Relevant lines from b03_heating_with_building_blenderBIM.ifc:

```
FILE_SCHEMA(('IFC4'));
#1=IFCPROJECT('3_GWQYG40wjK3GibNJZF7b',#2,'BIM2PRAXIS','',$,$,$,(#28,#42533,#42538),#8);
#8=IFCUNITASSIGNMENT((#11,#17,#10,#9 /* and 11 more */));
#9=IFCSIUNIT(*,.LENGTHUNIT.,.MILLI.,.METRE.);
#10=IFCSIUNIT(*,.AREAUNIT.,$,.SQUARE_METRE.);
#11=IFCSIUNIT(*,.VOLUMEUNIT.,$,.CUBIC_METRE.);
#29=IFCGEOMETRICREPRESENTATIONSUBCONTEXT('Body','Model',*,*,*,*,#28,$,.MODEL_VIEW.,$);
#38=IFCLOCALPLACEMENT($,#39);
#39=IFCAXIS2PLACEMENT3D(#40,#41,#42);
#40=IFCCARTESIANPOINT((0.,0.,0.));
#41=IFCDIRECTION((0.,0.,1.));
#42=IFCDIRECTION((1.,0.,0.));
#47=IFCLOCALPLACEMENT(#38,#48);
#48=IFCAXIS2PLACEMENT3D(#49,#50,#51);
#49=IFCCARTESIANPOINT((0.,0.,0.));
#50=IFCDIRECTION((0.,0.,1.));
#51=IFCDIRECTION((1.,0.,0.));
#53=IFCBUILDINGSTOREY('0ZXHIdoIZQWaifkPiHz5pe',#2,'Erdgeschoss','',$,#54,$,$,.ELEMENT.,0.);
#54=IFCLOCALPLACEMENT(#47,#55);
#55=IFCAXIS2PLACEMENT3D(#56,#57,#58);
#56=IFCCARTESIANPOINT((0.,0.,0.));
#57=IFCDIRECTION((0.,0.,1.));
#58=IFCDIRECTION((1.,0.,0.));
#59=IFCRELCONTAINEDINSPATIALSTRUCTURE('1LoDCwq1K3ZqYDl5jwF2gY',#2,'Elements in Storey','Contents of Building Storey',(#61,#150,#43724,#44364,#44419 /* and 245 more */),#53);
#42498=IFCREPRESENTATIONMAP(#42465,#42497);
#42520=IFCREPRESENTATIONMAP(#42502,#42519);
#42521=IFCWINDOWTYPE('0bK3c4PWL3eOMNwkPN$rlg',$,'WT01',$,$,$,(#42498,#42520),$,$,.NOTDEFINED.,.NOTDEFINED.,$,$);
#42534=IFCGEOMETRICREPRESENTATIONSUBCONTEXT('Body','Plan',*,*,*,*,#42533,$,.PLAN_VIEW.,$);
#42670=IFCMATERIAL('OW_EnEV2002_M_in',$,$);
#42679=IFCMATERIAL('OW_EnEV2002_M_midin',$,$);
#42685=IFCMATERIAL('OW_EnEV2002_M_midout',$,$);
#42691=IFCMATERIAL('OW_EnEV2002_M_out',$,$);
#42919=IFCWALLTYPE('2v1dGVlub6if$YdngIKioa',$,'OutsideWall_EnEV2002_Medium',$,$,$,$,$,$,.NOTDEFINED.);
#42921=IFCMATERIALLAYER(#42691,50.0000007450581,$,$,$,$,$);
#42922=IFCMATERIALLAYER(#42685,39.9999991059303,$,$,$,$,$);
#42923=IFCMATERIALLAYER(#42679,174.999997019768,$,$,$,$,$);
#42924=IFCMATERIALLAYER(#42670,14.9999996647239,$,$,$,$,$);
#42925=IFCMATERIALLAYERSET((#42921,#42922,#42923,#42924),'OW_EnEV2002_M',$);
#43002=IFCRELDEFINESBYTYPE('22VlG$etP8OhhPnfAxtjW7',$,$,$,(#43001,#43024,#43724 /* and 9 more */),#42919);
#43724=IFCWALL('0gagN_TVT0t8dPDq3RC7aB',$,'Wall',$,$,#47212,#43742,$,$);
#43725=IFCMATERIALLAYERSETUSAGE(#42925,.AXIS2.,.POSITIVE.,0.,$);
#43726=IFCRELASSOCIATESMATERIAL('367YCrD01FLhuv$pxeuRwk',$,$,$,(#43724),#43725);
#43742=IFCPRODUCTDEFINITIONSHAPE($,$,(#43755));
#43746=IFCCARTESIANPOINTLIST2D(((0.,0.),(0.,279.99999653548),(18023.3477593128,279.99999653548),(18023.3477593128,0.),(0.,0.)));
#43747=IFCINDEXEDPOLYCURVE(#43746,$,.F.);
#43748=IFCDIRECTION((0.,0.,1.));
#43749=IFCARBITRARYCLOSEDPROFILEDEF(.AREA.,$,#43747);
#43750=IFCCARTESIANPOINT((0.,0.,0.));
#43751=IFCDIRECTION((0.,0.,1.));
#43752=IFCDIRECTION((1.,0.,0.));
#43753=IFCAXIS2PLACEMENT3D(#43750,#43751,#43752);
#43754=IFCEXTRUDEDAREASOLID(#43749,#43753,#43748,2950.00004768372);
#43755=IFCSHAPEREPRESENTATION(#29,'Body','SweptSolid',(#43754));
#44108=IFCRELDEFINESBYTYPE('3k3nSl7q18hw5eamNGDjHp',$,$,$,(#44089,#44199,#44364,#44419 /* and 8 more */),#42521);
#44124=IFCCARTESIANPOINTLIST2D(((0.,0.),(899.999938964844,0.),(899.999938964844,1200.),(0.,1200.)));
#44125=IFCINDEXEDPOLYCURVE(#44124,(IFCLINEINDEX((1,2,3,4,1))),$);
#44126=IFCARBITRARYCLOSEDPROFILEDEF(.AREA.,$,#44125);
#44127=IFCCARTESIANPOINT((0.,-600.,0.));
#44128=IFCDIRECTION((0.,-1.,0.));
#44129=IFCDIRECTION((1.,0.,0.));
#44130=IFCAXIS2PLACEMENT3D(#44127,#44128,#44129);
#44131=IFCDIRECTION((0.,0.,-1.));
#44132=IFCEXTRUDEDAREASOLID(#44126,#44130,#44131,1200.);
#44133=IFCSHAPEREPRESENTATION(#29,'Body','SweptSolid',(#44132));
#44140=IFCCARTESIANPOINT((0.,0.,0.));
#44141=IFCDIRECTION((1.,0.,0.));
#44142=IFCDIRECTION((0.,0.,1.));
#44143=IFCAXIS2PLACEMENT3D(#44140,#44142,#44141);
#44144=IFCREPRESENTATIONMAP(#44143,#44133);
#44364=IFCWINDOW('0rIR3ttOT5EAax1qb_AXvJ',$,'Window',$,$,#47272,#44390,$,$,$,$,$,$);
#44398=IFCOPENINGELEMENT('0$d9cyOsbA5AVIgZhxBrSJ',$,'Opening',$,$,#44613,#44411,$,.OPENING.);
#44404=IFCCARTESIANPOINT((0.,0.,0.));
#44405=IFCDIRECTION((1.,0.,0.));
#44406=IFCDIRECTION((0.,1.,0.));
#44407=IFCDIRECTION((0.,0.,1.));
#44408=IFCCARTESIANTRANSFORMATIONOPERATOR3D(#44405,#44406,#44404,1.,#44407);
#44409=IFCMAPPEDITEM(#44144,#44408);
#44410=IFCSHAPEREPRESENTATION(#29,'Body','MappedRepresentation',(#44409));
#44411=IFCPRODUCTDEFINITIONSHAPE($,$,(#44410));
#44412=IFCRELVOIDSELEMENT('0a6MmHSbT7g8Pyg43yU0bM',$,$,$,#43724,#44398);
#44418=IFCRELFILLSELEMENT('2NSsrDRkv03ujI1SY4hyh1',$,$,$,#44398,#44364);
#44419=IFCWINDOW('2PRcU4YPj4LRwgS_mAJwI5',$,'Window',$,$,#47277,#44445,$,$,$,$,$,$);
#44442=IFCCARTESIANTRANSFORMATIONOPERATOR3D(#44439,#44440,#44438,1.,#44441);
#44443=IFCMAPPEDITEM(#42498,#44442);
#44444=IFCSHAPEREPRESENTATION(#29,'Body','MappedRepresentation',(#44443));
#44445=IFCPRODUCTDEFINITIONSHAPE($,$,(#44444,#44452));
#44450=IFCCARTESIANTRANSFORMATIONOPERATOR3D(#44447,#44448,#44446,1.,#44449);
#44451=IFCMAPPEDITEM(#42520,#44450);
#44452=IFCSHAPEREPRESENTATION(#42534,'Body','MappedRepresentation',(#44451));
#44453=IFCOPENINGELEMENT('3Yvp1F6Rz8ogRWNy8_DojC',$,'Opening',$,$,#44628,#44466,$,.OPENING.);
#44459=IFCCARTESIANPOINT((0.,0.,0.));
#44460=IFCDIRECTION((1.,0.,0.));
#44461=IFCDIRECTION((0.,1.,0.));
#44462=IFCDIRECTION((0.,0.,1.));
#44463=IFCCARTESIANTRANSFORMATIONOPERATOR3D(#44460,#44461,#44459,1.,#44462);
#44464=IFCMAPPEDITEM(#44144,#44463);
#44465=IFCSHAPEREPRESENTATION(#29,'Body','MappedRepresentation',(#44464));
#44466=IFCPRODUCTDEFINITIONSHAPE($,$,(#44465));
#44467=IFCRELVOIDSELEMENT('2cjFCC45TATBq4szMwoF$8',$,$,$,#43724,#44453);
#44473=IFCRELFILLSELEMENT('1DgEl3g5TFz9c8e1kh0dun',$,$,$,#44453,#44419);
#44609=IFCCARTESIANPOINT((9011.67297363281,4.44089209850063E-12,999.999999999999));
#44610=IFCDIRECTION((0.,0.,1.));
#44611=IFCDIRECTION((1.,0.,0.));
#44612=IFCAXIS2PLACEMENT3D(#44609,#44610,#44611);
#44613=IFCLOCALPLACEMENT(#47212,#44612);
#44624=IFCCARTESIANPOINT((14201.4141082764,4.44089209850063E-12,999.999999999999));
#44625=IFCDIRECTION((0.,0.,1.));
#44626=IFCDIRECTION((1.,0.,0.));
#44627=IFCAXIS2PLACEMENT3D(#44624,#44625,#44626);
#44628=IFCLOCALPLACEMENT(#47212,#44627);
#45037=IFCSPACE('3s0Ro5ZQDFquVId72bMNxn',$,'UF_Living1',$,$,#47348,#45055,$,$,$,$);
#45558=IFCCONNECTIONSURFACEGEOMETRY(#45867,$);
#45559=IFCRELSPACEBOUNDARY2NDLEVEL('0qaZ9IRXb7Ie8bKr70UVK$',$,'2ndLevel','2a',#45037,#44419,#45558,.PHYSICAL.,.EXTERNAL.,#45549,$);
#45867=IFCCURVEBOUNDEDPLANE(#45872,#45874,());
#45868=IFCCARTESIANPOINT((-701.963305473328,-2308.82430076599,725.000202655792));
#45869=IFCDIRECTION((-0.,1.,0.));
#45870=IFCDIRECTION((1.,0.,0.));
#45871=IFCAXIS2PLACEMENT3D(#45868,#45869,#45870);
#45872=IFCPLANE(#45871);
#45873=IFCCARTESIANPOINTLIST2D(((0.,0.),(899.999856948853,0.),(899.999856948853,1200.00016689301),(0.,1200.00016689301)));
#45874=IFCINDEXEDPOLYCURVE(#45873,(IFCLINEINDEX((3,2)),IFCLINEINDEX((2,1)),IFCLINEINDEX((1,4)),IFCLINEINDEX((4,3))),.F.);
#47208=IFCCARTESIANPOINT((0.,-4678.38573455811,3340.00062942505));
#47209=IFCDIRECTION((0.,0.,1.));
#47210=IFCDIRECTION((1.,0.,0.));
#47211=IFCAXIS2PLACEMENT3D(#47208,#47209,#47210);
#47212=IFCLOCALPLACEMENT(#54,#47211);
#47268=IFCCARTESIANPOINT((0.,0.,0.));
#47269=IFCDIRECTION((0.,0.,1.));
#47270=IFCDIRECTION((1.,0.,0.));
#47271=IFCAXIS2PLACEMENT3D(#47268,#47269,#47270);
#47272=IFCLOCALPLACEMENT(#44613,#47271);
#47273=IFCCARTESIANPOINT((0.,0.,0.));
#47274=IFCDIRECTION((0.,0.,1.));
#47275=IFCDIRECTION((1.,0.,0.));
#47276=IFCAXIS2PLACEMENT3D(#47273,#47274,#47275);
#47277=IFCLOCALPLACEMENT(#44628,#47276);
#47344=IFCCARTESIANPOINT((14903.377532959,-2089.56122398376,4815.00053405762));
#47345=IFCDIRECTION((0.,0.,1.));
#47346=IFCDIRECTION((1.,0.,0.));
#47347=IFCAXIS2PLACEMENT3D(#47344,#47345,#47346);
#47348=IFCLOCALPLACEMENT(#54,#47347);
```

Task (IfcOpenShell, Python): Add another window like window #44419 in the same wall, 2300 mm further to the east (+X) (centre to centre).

```python
import numpy as np
import ifcopenshell
import ifcopenshell.api.feature
import ifcopenshell.api.geometry
import ifcopenshell.api.root
import ifcopenshell.geom
import ifcopenshell.util.element
import ifcopenshell.util.placement
import ifcopenshell.util.shape
import ifcopenshell.util.unit

model = ifcopenshell.open("b03_heating_with_building_blenderBIM.ifc")
unit_scale = ifcopenshell.util.unit.calculate_unit_scale(model)
settings = ifcopenshell.geom.settings()


def volume(element):
    """Net volume in cubic metres, openings subtracted."""
    shape = ifcopenshell.geom.create_shape(settings, element)
    return ifcopenshell.util.shape.get_volume(shape.geometry)


window = model.by_guid("2PRcU4YPj4LRwgS_mAJwI5")
opening = window.FillsVoids[0].RelatingOpeningElement
wall = opening.VoidsElements[0].RelatingBuildingElement
before = volume(wall)
shift = ifcopenshell.util.placement.get_local_placement(wall.ObjectPlacement)[:3, 0] * 2.3 / unit_scale

# copy_class copies the void relationship, type, container and properties, but no geometry.
new_opening = ifcopenshell.api.root.copy_class(model, product=opening)
new_opening.Representation = ifcopenshell.util.element.copy_deep(
    model, opening.Representation, exclude=["IfcGeometricRepresentationContext", "IfcRepresentationMap"]
)
new_window = ifcopenshell.api.root.copy_class(model, product=window)
new_window.Representation = ifcopenshell.util.element.copy_deep(
    model, window.Representation, exclude=["IfcGeometricRepresentationContext", "IfcRepresentationMap"]
)
ifcopenshell.api.feature.add_filling(model, opening=new_opening, element=new_window)

for old, new in ((opening, new_opening), (window, new_window)):
    matrix = ifcopenshell.util.placement.get_local_placement(old.ObjectPlacement)
    matrix[:3, 3] += shift
    ifcopenshell.api.geometry.edit_object_placement(model, product=new, matrix=matrix, is_si=False)

# The copied space boundaries still share their surfaces with the original.
for rel in new_window.ProvidesBoundaries:
    if rel.ConnectionGeometry:
        rel.ConnectionGeometry = ifcopenshell.util.element.copy_deep(model, rel.ConnectionGeometry)

# Space boundary surfaces are stored in each space's coordinates; move them too.
for rel in new_window.ProvidesBoundaries:
    if not rel.ConnectionGeometry:
        continue
    surface = rel.ConnectionGeometry.SurfaceOnRelatingElement.BasisSurface
    space_matrix = ifcopenshell.util.placement.get_local_placement(rel.RelatingSpace.ObjectPlacement)
    point = np.array(surface.Position.Location.Coordinates) + space_matrix[:3, :3].T @ shift
    surface.Position = model.createIfcAxis2Placement3D(
        model.createIfcCartesianPoint(point.tolist()), surface.Position.Axis, surface.Position.RefDirection
    )

after = volume(wall)

print(f"wall volume {before:.3f} -> {after:.3f} m3")

model.write("b03_heating_with_building_blenderBIM_rev.ifc")
```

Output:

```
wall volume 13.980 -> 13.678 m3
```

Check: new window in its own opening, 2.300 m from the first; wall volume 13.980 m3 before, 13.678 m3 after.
